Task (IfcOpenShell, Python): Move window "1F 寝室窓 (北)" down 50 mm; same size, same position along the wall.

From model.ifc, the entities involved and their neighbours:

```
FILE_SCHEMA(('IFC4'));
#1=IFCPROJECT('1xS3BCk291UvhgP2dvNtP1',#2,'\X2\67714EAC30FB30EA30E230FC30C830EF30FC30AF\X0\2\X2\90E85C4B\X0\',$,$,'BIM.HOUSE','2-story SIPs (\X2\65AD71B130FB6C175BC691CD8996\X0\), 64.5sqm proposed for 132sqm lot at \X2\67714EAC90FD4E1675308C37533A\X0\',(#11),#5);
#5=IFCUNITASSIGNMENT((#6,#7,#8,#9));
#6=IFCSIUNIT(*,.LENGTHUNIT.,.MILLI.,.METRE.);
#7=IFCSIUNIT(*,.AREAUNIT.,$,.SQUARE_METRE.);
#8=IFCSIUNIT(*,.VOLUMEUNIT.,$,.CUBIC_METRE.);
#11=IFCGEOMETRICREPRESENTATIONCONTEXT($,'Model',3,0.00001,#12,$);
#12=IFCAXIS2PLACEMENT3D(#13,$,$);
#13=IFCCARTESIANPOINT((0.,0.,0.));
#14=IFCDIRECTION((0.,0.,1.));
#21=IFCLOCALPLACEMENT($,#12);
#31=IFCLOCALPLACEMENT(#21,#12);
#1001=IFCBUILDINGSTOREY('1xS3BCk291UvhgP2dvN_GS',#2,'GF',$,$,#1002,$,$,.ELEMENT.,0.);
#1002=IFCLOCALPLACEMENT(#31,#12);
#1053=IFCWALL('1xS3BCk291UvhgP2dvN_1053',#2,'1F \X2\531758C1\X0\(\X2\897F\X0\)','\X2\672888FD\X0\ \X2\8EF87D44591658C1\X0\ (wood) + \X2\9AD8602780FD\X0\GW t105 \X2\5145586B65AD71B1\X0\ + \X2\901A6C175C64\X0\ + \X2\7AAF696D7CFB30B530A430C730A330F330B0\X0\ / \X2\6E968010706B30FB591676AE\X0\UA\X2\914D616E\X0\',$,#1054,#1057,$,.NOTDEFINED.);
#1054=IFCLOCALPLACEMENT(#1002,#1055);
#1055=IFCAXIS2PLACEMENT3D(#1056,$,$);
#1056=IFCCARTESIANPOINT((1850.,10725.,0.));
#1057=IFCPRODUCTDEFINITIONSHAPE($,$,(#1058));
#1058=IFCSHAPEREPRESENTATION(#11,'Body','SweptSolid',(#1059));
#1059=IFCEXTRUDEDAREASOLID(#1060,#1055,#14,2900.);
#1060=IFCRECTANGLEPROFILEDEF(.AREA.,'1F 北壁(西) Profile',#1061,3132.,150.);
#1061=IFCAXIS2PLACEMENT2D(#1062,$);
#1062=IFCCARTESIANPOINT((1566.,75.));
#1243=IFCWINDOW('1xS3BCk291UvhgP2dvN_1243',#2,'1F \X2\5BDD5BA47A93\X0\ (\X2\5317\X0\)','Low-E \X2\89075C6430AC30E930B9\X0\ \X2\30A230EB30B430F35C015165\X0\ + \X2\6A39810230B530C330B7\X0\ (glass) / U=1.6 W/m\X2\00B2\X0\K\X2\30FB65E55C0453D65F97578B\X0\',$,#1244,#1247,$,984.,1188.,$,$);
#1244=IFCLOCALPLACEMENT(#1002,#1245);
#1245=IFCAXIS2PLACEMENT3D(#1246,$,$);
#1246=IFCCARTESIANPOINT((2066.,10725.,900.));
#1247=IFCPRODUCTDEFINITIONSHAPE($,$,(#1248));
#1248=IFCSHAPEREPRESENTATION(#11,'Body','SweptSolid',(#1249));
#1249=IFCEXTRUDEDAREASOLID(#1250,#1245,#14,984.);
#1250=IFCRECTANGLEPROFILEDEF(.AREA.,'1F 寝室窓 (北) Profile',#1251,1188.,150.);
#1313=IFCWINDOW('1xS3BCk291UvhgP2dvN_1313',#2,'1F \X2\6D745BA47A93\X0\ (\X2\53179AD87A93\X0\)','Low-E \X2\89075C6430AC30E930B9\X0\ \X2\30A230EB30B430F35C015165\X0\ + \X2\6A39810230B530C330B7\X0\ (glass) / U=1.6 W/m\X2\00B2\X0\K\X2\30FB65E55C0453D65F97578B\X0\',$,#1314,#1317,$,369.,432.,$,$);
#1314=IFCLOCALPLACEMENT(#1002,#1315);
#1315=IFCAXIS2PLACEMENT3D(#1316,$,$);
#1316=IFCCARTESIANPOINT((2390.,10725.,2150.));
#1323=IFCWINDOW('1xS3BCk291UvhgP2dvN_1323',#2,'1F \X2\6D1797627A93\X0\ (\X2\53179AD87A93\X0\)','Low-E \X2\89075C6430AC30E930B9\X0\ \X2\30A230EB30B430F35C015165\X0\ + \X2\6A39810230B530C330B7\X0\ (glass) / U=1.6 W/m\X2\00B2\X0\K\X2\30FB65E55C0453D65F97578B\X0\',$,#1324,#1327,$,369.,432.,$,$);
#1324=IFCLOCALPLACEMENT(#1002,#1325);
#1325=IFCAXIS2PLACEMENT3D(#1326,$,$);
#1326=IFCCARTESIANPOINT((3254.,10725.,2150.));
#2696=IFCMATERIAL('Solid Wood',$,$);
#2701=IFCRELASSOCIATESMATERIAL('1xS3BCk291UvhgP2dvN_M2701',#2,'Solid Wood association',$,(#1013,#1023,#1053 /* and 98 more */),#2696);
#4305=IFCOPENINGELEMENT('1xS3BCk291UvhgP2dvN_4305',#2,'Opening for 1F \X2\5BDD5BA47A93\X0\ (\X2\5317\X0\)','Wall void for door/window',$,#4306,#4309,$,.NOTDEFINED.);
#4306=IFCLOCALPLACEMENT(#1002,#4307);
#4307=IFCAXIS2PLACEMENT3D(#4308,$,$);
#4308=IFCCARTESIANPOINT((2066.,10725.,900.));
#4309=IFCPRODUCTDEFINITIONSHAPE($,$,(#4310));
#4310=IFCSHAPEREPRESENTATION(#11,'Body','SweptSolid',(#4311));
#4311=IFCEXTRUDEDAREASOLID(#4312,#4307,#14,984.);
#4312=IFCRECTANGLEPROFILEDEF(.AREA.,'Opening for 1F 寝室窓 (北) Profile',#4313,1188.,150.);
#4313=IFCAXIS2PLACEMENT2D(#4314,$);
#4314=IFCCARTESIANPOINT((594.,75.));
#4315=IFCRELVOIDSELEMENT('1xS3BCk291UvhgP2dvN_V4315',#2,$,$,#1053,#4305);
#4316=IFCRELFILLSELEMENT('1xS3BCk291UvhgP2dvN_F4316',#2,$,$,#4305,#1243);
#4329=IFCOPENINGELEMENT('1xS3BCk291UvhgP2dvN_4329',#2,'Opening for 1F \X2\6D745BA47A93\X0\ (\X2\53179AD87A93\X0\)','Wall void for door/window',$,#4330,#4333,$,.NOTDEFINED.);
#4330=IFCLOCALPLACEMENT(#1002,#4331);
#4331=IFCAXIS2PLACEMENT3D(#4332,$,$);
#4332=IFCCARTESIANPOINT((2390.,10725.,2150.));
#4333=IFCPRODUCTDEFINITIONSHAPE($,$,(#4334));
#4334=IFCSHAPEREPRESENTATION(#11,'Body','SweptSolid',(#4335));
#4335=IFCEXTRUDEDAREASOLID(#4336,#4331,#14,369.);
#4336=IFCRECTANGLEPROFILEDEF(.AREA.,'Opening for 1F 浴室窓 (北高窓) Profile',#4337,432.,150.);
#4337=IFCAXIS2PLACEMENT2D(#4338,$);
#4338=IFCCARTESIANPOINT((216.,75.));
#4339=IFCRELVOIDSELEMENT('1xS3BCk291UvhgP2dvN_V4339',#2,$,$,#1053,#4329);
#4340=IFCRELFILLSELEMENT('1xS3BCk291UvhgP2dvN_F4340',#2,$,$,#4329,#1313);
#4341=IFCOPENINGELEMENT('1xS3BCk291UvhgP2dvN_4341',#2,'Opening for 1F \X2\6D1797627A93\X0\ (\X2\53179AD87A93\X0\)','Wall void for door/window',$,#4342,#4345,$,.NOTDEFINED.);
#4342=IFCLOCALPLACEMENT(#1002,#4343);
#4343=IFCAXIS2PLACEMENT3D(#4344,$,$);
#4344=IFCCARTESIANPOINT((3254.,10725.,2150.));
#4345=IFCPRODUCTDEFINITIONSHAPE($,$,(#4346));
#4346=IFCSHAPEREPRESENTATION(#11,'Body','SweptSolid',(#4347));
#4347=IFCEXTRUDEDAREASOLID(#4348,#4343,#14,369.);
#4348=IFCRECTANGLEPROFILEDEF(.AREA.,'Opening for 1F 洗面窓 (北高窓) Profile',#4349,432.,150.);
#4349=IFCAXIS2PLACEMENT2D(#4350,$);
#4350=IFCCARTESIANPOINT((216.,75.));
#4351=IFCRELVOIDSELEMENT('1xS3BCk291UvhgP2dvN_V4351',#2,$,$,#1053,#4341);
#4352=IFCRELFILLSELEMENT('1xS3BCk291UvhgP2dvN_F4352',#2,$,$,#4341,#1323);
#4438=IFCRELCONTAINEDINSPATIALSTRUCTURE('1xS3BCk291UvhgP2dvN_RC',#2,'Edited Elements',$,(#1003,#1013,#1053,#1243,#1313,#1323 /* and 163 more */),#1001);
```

```python
import numpy as np
import ifcopenshell
import ifcopenshell.api.geometry
import ifcopenshell.util.placement
import ifcopenshell.util.unit

model = ifcopenshell.open("model.ifc")
unit_scale = ifcopenshell.util.unit.calculate_unit_scale(model)

window = model.by_guid("1xS3BCk291UvhgP2dvN_1243")
opening = window.FillsVoids[0].RelatingOpeningElement
dz = -50.0

shift = np.array([0.0, 0.0, dz])
# The window is not placed relative to its opening, so move both.
for product in (opening, window):
    matrix = ifcopenshell.util.placement.get_local_placement(product.ObjectPlacement)
    matrix[:3, 3] += shift
    ifcopenshell.api.geometry.edit_object_placement(model, product=product, matrix=matrix, is_si=False)

print(f"moved by {dz * unit_scale:+.3f} m")

model.write("model_edited.ifc")
```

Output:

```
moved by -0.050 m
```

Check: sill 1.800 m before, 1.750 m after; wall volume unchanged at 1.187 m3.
